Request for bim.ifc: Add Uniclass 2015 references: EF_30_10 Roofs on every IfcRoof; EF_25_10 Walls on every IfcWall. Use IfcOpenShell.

First a look at what the model holds.

```python
import ifcopenshell

model = ifcopenshell.open("bim.ifc")
print(model.schema)
print("classifications:", [c.Name for c in model.by_type("IfcClassification")])
for ifc_class in ("IfcDoor", "IfcRoof", "IfcStair", "IfcWall", "IfcWindow"):
    print(ifc_class, len(model.by_type(ifc_class)))
```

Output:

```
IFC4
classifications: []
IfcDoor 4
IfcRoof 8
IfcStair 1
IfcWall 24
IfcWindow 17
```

```python
import ifcopenshell
import ifcopenshell.api.classification

model = ifcopenshell.open("bim.ifc")

system = ifcopenshell.api.classification.add_classification(model, classification="Uniclass 2015")

codes = {
    "IfcRoof": ("EF_30_10", "Roofs"),
    "IfcWall": ("EF_25_10", "Walls"),
}
for ifc_class, (code, name) in codes.items():
    products = model.by_type(ifc_class)
    ifcopenshell.api.classification.add_reference(
        model, products=products, classification=system, identification=code, name=name
    )
    print(code, len(products))

model.write("bim_rev.ifc")
```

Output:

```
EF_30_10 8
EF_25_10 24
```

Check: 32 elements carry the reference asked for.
